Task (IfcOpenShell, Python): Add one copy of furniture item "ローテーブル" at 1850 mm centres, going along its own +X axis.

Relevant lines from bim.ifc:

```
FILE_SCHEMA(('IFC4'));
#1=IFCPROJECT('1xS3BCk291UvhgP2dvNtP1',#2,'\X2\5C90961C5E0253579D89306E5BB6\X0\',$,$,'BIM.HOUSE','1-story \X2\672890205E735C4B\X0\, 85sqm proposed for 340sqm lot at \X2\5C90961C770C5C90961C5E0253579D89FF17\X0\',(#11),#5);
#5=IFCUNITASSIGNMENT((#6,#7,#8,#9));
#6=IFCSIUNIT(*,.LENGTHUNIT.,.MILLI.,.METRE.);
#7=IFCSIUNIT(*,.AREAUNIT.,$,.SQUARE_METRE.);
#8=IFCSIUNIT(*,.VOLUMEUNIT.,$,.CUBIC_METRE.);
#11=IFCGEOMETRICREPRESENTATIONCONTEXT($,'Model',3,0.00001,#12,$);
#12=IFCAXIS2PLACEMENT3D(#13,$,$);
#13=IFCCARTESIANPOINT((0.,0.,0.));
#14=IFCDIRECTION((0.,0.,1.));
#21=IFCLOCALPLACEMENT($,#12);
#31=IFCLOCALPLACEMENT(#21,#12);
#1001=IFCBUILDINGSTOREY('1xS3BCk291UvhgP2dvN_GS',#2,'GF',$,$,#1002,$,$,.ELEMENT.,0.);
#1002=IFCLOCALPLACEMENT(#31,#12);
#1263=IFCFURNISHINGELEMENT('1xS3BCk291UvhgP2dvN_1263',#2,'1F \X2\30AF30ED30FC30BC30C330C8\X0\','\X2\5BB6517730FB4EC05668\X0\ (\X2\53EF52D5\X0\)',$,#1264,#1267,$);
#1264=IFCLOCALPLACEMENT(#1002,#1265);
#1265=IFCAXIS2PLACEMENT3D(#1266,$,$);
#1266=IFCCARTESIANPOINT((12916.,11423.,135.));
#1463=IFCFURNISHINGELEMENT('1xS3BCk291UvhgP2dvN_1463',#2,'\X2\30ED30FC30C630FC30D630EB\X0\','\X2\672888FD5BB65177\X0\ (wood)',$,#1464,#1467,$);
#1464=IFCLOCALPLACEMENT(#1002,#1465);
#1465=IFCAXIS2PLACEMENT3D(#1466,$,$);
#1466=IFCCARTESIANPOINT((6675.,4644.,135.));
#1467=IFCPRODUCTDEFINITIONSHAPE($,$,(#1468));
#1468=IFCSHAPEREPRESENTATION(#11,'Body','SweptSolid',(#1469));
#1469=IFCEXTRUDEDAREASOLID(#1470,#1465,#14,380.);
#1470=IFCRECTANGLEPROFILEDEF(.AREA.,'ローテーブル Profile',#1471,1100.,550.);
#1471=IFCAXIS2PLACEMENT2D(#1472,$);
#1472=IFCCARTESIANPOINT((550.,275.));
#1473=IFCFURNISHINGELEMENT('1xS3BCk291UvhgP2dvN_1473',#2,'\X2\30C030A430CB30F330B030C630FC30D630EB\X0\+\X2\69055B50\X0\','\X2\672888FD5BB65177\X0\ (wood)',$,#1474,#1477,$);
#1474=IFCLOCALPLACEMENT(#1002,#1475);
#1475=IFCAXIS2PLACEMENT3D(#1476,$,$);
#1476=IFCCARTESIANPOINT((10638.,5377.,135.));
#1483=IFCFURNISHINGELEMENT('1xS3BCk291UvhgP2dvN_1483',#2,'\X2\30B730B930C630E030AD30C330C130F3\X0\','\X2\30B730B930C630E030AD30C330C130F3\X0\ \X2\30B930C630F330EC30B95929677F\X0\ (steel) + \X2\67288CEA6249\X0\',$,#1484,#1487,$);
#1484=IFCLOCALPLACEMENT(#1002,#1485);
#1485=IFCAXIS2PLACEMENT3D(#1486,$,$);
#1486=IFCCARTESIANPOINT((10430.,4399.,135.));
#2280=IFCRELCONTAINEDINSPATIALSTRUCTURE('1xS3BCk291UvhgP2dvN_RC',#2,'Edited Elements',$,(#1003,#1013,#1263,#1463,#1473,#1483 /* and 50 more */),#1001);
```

```python
import ifcopenshell
import ifcopenshell.api.geometry
import ifcopenshell.api.root
import ifcopenshell.util.element
import ifcopenshell.util.placement

model = ifcopenshell.open("bim.ifc")


def reuse_history(source, copy):
    """copy_class also copies each property set's owner history, people and application; keep the originals."""
    for rel in copy.IsDefinedBy:
        if rel.is_a("IfcRelDefinesByProperties") and (history := rel.RelatingPropertyDefinition.OwnerHistory):
            rel.RelatingPropertyDefinition.OwnerHistory = source.OwnerHistory
            ifcopenshell.util.element.remove_deep2(model, history)


source = model.by_guid("1xS3BCk291UvhgP2dvN_1463")
base = ifcopenshell.util.placement.get_local_placement(source.ObjectPlacement)
step = base[:3, 0] * 1850.0

for i in range(1, 2):
    copy = ifcopenshell.api.root.copy_class(model, product=source)
    copy.Representation = ifcopenshell.util.element.copy_deep(
        model, source.Representation, exclude=["IfcGeometricRepresentationContext", "IfcRepresentationMap"]
    )
    reuse_history(source, copy)
    matrix = base.copy()
    matrix[:3, 3] += i * step
    print("added at", matrix[:3, 3].round(3) + 0.0)
    ifcopenshell.api.geometry.edit_object_placement(model, product=copy, matrix=matrix, is_si=False)

model.write("bim_v2.ifc")
```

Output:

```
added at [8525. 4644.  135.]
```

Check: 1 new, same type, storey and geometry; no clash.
